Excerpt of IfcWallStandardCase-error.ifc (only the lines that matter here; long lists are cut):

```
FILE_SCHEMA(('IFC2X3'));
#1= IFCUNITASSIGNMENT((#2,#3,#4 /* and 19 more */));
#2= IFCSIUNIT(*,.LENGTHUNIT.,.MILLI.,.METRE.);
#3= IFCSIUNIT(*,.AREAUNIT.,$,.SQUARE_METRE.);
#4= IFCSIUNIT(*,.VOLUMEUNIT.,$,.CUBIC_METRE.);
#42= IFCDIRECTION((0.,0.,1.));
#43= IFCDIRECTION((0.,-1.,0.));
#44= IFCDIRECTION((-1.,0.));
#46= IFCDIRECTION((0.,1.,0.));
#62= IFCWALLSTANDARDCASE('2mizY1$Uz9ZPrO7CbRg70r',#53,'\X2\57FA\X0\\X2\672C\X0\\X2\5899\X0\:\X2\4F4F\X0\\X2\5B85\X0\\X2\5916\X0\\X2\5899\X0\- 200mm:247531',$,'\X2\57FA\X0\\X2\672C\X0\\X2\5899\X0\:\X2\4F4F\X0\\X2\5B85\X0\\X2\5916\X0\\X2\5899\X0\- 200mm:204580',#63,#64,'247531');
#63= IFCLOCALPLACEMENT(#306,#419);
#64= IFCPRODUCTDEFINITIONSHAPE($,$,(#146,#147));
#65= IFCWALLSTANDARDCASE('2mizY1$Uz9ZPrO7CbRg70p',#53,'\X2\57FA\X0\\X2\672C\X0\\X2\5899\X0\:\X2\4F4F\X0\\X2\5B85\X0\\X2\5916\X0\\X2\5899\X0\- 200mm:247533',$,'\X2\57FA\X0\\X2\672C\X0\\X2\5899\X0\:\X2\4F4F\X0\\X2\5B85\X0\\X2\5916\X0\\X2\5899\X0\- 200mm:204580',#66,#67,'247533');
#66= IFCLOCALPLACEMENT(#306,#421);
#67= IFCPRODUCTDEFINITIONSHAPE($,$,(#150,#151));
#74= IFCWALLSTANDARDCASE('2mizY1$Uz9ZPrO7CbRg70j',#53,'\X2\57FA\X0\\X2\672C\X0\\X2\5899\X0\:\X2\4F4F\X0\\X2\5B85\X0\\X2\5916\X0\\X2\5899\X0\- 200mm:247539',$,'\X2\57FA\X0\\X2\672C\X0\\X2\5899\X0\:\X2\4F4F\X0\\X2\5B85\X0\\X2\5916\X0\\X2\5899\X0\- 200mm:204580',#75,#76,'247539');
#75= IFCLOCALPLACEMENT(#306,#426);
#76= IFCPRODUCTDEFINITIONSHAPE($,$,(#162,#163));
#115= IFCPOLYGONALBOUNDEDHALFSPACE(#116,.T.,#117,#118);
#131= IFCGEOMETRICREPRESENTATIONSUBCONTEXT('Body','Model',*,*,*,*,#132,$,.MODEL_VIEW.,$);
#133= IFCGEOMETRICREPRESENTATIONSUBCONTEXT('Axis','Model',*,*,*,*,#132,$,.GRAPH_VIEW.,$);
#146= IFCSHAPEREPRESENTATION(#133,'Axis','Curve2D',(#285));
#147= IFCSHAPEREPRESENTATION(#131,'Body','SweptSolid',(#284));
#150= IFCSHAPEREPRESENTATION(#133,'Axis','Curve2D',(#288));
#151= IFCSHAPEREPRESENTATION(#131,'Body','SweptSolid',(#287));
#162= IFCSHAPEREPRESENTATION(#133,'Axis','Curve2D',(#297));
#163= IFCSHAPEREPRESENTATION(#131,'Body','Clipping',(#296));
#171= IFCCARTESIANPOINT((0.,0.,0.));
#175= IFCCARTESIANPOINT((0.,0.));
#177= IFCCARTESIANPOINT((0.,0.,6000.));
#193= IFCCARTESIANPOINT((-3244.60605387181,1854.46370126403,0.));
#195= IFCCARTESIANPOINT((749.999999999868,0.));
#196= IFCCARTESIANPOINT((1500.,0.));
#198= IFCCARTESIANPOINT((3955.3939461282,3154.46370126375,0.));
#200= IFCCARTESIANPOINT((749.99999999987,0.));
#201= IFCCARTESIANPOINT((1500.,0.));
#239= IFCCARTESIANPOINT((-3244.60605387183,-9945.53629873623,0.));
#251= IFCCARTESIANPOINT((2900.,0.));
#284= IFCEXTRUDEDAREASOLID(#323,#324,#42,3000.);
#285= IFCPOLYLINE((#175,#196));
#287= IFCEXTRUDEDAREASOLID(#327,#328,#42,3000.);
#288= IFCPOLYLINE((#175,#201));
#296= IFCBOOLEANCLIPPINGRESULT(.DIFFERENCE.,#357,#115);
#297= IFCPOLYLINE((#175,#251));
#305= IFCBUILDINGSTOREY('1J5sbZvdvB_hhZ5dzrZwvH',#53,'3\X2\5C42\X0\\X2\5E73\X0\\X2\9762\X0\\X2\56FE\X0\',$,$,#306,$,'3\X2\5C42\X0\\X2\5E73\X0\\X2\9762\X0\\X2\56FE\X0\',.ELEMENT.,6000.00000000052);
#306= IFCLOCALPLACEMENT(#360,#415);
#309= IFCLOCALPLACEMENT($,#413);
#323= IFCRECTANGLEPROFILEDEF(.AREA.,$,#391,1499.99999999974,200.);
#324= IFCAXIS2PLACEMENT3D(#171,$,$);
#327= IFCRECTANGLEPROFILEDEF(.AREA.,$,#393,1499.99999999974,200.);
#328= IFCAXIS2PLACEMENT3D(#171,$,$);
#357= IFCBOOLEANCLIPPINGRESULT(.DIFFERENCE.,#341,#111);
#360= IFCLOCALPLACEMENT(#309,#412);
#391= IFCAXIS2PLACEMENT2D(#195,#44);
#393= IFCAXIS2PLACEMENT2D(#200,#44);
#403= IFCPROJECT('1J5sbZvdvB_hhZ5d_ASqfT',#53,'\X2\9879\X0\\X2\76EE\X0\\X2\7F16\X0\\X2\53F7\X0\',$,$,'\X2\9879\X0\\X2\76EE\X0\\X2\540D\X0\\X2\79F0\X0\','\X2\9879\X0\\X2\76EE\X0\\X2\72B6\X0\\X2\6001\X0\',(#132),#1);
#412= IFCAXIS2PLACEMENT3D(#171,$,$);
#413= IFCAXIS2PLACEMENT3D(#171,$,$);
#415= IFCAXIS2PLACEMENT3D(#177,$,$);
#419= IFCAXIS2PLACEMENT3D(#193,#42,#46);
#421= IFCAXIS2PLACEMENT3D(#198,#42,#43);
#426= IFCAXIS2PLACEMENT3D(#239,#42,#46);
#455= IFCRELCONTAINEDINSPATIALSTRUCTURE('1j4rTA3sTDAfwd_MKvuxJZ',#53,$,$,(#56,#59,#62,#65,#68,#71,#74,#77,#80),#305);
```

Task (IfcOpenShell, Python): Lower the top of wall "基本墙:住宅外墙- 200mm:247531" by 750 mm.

```python
import ifcopenshell
import ifcopenshell.geom
import ifcopenshell.util.representation
import ifcopenshell.util.shape

model = ifcopenshell.open("IfcWallStandardCase-error.ifc")
settings = ifcopenshell.geom.settings()


def volume(element):
    """Net volume in cubic metres, openings subtracted."""
    shape = ifcopenshell.geom.create_shape(settings, element)
    return ifcopenshell.util.shape.get_volume(shape.geometry)


wall = model.by_guid("2mizY1$Uz9ZPrO7CbRg70r")
before = volume(wall)

body = ifcopenshell.util.representation.get_representation(wall, "Model", "Body")
solid = body.Items[0]
old_height = solid.Depth
solid.Depth -= 750.0
after = volume(wall)

print(f"height {old_height:g} -> {solid.Depth:g}, volume {before:.3f} -> {after:.3f} m3")

model.write("IfcWallStandardCase-error_updated.ifc")
```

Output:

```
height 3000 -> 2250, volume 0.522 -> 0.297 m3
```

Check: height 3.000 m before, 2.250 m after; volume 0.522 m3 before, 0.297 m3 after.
